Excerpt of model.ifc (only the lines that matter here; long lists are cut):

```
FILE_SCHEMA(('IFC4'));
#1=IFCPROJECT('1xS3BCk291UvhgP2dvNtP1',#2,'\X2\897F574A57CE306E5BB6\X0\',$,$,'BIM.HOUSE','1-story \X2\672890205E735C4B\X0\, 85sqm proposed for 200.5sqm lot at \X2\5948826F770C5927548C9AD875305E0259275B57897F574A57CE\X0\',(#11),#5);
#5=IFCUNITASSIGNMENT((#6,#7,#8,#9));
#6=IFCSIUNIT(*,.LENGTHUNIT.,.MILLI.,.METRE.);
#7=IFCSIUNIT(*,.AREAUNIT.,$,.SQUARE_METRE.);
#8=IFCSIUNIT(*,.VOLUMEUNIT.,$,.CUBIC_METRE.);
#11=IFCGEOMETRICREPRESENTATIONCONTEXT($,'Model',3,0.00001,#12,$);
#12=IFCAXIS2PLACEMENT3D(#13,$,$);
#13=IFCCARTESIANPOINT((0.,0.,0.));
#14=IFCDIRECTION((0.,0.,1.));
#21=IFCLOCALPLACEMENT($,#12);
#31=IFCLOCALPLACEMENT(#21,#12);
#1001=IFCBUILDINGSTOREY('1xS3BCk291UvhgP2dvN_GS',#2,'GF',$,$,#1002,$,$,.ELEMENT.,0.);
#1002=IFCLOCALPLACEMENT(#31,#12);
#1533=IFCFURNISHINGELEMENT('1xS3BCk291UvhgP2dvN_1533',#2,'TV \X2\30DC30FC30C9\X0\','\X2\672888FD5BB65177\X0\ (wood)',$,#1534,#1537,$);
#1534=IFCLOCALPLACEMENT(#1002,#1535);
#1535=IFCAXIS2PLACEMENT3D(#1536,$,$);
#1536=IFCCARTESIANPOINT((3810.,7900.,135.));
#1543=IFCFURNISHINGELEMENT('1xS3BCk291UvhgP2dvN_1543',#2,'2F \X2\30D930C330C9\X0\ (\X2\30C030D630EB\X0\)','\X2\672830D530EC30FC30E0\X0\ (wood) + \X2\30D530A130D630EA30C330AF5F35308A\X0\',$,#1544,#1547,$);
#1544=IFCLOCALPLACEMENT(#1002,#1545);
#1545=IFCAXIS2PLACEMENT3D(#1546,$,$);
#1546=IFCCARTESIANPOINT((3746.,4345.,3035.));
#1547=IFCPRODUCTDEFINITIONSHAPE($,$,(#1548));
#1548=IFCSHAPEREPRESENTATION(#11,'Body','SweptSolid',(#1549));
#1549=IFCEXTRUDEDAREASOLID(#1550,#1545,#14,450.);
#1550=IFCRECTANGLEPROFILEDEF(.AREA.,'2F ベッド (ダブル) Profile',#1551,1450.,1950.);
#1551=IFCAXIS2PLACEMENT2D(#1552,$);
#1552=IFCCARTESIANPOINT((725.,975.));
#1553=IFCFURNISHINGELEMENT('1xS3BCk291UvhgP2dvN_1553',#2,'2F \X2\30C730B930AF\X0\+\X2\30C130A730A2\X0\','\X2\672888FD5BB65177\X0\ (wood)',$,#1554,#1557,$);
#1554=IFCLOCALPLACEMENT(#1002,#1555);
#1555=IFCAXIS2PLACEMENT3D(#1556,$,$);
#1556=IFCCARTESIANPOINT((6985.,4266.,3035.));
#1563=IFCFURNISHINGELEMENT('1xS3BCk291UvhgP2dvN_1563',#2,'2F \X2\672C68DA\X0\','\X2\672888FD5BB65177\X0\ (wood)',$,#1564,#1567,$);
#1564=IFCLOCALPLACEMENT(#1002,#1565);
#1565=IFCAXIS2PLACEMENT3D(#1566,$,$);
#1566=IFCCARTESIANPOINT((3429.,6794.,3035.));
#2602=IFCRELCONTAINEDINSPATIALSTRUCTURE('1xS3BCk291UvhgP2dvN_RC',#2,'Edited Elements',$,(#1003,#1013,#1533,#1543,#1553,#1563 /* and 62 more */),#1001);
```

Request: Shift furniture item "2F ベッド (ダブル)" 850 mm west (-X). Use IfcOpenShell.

```python
import ifcopenshell
import ifcopenshell.api.geometry
import ifcopenshell.util.placement
import ifcopenshell.util.unit

model = ifcopenshell.open("model.ifc")
unit_scale = ifcopenshell.util.unit.calculate_unit_scale(model)

item = model.by_guid("1xS3BCk291UvhgP2dvN_1543")
matrix = ifcopenshell.util.placement.get_local_placement(item.ObjectPlacement)
matrix[0, 3] -= 0.85 / unit_scale
ifcopenshell.api.geometry.edit_object_placement(model, product=item, matrix=matrix, is_si=False)

print(ifcopenshell.util.placement.get_local_placement(item.ObjectPlacement).round(3) + 0.0)

model.write("model_rev.ifc")
```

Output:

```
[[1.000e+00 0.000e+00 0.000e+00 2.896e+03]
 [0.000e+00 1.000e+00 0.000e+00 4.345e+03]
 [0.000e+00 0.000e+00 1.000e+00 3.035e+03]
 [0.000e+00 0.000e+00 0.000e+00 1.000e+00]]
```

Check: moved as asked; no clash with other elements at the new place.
